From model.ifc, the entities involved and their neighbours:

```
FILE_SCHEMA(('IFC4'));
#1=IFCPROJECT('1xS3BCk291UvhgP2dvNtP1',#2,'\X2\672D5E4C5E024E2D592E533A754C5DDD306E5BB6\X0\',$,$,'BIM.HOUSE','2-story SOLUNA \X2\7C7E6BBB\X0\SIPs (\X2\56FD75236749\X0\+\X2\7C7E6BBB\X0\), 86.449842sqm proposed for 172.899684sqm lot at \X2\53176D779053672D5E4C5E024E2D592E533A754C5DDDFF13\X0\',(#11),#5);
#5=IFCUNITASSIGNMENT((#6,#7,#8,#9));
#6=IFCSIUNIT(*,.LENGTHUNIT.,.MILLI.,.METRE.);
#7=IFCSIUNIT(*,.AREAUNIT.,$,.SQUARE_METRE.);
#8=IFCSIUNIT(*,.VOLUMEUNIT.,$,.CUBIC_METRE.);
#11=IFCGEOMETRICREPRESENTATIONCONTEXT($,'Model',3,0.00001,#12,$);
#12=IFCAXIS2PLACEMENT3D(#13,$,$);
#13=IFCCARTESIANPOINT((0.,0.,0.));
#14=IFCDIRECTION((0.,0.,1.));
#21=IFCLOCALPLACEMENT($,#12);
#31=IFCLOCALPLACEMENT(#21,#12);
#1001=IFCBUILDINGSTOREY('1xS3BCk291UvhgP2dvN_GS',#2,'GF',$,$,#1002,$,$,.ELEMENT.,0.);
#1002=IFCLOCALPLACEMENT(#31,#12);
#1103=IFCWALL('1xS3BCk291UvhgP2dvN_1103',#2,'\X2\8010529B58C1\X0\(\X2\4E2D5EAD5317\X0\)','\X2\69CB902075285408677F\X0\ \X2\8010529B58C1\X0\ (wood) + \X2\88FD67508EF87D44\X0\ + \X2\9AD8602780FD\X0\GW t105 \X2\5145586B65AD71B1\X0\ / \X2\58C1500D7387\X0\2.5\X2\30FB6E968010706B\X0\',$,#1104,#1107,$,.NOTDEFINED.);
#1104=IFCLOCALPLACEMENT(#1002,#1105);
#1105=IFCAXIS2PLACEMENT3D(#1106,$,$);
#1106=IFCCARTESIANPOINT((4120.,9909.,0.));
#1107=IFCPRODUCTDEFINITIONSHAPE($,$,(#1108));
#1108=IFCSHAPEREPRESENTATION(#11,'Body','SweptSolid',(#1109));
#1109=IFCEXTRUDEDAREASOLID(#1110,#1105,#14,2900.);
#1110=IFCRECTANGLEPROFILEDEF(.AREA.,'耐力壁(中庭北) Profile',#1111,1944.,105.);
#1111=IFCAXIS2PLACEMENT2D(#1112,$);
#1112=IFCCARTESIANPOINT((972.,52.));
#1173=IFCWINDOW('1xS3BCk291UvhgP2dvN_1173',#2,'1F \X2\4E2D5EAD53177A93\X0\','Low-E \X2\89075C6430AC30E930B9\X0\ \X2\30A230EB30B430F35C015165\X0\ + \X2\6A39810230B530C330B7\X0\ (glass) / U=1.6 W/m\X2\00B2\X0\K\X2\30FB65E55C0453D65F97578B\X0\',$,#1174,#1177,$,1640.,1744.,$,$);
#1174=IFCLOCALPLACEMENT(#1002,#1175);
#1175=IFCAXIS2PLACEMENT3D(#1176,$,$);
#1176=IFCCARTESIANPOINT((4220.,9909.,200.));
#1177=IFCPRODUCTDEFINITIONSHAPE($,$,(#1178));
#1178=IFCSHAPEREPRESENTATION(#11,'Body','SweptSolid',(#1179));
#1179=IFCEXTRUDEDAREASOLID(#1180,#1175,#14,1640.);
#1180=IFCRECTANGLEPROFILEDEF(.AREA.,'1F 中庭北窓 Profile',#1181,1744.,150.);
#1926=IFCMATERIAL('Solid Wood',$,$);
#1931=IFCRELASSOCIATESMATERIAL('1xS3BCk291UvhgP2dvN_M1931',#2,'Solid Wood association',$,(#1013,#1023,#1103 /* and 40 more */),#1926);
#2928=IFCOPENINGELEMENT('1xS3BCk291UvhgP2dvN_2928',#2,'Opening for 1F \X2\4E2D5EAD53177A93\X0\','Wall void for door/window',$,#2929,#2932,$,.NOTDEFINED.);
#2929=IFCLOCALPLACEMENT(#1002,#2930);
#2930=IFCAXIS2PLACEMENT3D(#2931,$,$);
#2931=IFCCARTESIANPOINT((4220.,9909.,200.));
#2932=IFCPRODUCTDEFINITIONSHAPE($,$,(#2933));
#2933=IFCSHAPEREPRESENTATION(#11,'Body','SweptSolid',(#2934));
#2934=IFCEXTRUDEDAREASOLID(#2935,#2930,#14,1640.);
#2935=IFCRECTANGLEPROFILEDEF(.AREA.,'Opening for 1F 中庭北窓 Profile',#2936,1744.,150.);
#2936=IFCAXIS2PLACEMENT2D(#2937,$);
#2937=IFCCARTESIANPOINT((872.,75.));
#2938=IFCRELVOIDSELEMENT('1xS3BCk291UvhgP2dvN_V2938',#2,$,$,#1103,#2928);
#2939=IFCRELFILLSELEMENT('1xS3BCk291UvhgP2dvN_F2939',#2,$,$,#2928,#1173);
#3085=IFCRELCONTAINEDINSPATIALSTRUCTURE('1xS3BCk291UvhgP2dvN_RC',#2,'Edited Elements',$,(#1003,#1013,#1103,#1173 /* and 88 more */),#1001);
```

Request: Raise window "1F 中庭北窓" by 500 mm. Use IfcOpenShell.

```python
import numpy as np
import ifcopenshell
import ifcopenshell.api.geometry
import ifcopenshell.util.placement
import ifcopenshell.util.unit

model = ifcopenshell.open("model.ifc")
unit_scale = ifcopenshell.util.unit.calculate_unit_scale(model)

window = model.by_guid("1xS3BCk291UvhgP2dvN_1173")
opening = window.FillsVoids[0].RelatingOpeningElement
dz = 500.0

shift = np.array([0.0, 0.0, dz])
# The window is not placed relative to its opening, so move both.
for product in (opening, window):
    matrix = ifcopenshell.util.placement.get_local_placement(product.ObjectPlacement)
    matrix[:3, 3] += shift
    ifcopenshell.api.geometry.edit_object_placement(model, product=product, matrix=matrix, is_si=False)

print(f"moved by {dz * unit_scale:+.3f} m")

model.write("model_v2.ifc")
```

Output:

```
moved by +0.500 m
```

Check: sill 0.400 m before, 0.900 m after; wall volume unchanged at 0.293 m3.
